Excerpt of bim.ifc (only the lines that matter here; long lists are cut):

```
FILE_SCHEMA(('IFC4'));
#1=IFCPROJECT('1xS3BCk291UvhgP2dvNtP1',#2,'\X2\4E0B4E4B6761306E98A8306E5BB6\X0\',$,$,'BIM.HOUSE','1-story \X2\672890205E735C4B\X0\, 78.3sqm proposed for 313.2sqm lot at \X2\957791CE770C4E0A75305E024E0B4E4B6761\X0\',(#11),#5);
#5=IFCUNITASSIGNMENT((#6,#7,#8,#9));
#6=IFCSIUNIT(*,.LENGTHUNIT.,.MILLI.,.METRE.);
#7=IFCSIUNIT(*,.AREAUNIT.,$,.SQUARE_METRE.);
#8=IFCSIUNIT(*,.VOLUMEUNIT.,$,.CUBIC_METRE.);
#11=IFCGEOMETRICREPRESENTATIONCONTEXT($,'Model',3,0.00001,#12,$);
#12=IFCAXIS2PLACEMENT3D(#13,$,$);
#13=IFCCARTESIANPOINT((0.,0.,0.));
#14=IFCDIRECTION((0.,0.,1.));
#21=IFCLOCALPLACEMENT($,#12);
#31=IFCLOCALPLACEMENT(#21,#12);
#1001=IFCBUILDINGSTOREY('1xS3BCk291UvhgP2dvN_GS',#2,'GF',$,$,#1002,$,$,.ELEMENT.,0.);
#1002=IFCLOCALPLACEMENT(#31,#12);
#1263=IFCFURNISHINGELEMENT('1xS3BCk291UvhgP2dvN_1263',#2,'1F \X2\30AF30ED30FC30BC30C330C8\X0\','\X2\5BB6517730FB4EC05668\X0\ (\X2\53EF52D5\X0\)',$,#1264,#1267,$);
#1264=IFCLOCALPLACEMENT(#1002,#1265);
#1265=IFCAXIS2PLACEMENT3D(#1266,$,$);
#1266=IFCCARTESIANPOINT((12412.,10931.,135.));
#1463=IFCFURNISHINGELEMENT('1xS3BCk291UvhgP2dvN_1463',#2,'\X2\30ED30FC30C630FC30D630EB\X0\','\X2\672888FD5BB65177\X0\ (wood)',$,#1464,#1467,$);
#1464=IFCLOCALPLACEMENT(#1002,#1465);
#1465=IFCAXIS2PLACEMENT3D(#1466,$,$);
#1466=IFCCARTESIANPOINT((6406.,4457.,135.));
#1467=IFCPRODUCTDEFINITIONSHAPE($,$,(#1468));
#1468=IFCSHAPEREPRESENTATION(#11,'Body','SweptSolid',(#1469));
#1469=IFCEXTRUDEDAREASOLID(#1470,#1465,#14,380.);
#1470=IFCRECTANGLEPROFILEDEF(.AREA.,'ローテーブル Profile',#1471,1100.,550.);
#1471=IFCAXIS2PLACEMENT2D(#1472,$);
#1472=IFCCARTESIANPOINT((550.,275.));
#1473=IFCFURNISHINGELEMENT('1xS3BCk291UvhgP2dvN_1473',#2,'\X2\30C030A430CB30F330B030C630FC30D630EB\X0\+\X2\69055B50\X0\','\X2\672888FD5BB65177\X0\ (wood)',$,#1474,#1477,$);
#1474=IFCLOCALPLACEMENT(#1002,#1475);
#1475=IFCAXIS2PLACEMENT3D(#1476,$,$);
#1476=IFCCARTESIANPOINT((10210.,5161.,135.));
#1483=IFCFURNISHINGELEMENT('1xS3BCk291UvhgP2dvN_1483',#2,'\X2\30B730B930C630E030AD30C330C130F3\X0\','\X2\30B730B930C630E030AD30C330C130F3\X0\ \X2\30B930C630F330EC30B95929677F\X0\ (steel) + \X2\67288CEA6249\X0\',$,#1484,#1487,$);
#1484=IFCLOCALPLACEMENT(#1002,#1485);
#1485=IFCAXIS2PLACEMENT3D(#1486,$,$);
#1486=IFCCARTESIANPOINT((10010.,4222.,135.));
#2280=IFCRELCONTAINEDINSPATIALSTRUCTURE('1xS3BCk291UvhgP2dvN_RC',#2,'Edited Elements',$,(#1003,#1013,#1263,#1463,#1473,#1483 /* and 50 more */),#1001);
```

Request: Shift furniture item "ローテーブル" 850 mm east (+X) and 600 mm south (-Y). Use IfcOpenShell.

```python
import ifcopenshell
import ifcopenshell.api.geometry
import ifcopenshell.util.placement
import ifcopenshell.util.unit

model = ifcopenshell.open("bim.ifc")
unit_scale = ifcopenshell.util.unit.calculate_unit_scale(model)

item = model.by_id(1463)
matrix = ifcopenshell.util.placement.get_local_placement(item.ObjectPlacement)
matrix[0, 3] += 0.85 / unit_scale
matrix[1, 3] -= 0.6 / unit_scale
ifcopenshell.api.geometry.edit_object_placement(model, product=item, matrix=matrix, is_si=False)

print(ifcopenshell.util.placement.get_local_placement(item.ObjectPlacement).round(3) + 0.0)

model.write("bim-out.ifc")
```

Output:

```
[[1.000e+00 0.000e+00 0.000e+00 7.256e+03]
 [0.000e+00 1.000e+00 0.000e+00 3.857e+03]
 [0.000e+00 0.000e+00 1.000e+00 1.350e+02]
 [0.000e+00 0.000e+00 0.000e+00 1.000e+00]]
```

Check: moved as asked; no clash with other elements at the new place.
